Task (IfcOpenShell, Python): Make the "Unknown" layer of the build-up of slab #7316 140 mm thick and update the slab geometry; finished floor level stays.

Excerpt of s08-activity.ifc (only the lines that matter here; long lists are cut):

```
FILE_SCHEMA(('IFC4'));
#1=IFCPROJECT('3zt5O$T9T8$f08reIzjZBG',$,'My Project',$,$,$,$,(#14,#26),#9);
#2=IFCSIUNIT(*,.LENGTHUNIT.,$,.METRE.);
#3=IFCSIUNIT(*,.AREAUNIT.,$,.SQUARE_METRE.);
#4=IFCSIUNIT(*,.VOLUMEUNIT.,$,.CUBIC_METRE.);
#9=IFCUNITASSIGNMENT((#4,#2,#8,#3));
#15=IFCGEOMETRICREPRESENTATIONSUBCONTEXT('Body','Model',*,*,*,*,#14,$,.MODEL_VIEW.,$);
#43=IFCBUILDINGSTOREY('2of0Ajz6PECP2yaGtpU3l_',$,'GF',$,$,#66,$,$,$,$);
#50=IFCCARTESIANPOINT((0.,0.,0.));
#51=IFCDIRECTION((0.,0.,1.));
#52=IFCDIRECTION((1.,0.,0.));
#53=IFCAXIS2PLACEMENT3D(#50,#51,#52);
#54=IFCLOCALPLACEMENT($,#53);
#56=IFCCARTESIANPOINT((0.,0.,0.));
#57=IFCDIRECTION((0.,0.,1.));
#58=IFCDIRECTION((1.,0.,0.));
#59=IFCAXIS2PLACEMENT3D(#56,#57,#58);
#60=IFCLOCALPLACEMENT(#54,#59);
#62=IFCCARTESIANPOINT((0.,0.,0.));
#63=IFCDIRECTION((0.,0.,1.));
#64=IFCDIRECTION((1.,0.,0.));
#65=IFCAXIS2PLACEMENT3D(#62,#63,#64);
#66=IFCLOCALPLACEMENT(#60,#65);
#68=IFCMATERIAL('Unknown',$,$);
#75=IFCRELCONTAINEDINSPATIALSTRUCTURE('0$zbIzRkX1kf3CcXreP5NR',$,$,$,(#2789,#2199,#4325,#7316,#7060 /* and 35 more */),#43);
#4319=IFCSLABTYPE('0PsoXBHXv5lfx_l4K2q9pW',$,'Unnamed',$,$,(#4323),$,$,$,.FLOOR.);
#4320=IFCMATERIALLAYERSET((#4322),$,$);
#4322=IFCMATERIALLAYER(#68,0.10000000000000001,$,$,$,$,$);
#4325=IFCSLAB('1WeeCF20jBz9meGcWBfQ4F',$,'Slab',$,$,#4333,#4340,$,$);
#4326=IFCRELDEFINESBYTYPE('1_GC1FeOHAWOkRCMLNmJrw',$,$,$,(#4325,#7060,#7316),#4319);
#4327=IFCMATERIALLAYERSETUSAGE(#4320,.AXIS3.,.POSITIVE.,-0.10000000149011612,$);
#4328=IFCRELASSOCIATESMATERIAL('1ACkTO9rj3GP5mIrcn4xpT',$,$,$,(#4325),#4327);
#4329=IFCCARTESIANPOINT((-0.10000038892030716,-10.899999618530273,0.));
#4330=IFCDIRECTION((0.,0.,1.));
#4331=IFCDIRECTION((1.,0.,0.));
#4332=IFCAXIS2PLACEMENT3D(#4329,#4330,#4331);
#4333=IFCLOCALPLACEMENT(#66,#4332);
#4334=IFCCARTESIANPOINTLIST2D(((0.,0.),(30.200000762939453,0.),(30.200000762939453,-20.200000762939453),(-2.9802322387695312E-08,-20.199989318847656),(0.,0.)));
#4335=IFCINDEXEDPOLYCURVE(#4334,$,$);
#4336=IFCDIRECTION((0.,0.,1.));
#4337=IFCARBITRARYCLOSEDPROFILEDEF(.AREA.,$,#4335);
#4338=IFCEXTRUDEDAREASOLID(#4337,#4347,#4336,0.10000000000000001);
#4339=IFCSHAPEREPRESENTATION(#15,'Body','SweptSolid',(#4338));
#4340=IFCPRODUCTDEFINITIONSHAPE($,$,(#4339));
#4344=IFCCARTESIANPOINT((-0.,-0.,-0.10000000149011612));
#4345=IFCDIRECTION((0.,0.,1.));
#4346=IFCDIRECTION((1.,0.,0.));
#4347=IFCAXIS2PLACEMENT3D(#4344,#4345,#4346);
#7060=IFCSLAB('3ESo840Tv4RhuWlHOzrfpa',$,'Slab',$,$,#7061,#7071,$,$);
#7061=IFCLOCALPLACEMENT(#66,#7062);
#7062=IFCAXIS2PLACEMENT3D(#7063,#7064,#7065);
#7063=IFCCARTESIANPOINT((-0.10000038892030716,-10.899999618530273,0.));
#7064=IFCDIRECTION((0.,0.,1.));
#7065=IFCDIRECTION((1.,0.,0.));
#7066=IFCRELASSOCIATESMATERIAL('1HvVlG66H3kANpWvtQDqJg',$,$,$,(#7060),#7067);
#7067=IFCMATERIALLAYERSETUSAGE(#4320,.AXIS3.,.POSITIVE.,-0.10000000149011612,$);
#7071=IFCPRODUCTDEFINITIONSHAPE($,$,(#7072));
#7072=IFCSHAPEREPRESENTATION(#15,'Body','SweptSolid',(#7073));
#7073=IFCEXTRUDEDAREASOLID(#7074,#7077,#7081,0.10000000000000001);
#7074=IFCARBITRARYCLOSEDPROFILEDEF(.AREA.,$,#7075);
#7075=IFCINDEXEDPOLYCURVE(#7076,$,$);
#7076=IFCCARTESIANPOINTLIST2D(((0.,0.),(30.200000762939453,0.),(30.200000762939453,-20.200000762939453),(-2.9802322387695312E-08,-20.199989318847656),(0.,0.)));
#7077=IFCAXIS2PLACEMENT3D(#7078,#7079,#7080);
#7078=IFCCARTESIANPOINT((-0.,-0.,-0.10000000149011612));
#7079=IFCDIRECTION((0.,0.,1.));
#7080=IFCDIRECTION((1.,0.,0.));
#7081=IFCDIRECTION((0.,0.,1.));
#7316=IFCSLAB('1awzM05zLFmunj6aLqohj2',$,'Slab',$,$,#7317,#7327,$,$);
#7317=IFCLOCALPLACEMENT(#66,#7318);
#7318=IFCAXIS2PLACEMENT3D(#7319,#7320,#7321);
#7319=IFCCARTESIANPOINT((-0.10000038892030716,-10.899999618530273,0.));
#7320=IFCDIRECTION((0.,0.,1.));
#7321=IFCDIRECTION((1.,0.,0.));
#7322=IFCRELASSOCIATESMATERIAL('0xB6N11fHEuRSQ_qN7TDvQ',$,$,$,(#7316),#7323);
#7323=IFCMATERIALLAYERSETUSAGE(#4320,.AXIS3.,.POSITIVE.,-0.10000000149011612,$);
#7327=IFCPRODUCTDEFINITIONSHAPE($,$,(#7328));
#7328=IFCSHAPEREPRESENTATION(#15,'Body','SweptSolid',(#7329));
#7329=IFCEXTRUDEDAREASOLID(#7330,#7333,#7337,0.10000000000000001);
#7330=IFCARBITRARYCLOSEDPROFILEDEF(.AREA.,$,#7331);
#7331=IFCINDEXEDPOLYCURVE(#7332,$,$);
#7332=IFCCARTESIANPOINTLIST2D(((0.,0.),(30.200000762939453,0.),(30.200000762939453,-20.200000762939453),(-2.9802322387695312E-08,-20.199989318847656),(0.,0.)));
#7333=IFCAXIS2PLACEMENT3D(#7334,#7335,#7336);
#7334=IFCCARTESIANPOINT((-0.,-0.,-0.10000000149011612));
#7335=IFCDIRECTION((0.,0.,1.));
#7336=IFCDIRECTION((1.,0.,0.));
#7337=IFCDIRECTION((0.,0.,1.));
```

```python
import ifcopenshell
import ifcopenshell.util.element
import ifcopenshell.util.representation

model = ifcopenshell.open("s08-activity.ifc")

layer_set = model.by_id(4320)
layer = next(l for l in layer_set.MaterialLayers if l.Material and l.Material.Name == "Unknown")
change = 0.14 - layer.LayerThickness
layer.LayerThickness += change

# The layer set is shared, so every slab that uses it gets the new thickness.
slabs = [e for e in ifcopenshell.util.element.get_elements_by_material(model, layer_set) if e.is_a("IfcSlab")]
for slab in sorted(slabs, key=lambda e: e.id()):
    body = ifcopenshell.util.representation.get_representation(slab, "Model", "Body")
    solid = body.Items[0]
    old_depth = solid.Depth
    solid.Depth += change
    # Extruded upwards: lower the start of the extrusion so the top stays.
    x, y, z = solid.Position.Location.Coordinates
    solid.Position.Location = model.createIfcCartesianPoint((x, y, z - change))
    print(slab.id(), f"{old_depth:g} -> {solid.Depth:g}")

# The layers are counted up from the underside, which has moved.
for usage in {ifcopenshell.util.element.get_material(slab) for slab in slabs}:
    usage.OffsetFromReferenceLine -= change

model.write("s08-activity_rev.ifc")
```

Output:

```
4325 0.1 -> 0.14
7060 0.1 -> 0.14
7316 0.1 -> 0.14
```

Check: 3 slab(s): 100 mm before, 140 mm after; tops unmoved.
